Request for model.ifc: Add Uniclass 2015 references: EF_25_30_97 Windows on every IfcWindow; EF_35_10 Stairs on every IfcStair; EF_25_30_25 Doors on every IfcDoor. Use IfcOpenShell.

First a look at what the model holds.

```python
import ifcopenshell

model = ifcopenshell.open("model.ifc")
print(model.schema)
print("classifications:", [c.Name for c in model.by_type("IfcClassification")])
for ifc_class in ("IfcDoor", "IfcRoof", "IfcStair", "IfcWall", "IfcWindow"):
    print(ifc_class, len(model.by_type(ifc_class)))
```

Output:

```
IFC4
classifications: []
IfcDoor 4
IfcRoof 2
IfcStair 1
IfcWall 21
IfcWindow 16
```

```python
import ifcopenshell
import ifcopenshell.api.classification

model = ifcopenshell.open("model.ifc")

system = ifcopenshell.api.classification.add_classification(model, classification="Uniclass 2015")

codes = {
    "IfcWindow": ("EF_25_30_97", "Windows"),
    "IfcStair": ("EF_35_10", "Stairs"),
    "IfcDoor": ("EF_25_30_25", "Doors"),
}
for ifc_class, (code, name) in codes.items():
    products = model.by_type(ifc_class)
    ifcopenshell.api.classification.add_reference(
        model, products=products, classification=system, identification=code, name=name
    )
    print(code, len(products))

model.write("model_edited.ifc")
```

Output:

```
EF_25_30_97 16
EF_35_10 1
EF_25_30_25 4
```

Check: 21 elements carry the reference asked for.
